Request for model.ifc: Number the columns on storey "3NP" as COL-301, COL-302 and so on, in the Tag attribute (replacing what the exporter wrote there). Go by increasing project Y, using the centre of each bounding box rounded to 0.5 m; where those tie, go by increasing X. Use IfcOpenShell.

First a look at what the model holds.

```python
import ifcopenshell
import ifcopenshell.util.element
import ifcopenshell.util.placement

model = ifcopenshell.open("model.ifc")
print(model.schema)
storey = next(s for s in model.by_type("IfcBuildingStorey") if s.Name == "3NP")
columns = [e for e in ifcopenshell.util.element.get_decomposition(storey) if e.is_a("IfcColumn")]
for e in sorted(columns, key=lambda e: e.id()):
    origin = ifcopenshell.util.placement.get_local_placement(e.ObjectPlacement)[:3, 3]
    print(e.id(), e.Tag, e.Name, origin.round(2) + 0.0, sep=" | ")
```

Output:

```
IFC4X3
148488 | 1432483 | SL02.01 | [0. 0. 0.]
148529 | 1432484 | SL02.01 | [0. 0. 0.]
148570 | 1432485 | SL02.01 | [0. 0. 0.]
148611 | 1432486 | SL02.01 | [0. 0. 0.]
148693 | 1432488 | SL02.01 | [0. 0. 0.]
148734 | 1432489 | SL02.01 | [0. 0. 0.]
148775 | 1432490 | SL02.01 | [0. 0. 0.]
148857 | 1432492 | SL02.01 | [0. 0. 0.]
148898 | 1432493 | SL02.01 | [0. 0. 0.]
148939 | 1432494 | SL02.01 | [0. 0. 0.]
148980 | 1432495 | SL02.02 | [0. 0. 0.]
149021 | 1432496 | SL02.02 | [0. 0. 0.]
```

```python
import ifcopenshell
import ifcopenshell.geom
import ifcopenshell.util.element
import ifcopenshell.util.shape

model = ifcopenshell.open("model.ifc")
settings = ifcopenshell.geom.settings()
settings.set("use-world-coords", True)


def centre(element):
    shape = ifcopenshell.geom.create_shape(settings, element)
    return ifcopenshell.util.shape.get_bbox_centroid(shape.geometry)


storey = next(s for s in model.by_type("IfcBuildingStorey") if s.Name == "3NP")
columns = [e for e in ifcopenshell.util.element.get_decomposition(storey) if e.is_a("IfcColumn")]

# Insertion points can sit at a corner or the storey origin, so sort by the geometry (in metres).
centres = {e: centre(e) for e in columns}
columns.sort(key=lambda e: (round(centres[e][1] / 0.5), centres[e][0]))

for i, e in enumerate(columns, start=1):
    number = f"COL-3{i:02d}"
    e.Tag = number
    print(e.id(), number)

model.write("model-out.ifc")
```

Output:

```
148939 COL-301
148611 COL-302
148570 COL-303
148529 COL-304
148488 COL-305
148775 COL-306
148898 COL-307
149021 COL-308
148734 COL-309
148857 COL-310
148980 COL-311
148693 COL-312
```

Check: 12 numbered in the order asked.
